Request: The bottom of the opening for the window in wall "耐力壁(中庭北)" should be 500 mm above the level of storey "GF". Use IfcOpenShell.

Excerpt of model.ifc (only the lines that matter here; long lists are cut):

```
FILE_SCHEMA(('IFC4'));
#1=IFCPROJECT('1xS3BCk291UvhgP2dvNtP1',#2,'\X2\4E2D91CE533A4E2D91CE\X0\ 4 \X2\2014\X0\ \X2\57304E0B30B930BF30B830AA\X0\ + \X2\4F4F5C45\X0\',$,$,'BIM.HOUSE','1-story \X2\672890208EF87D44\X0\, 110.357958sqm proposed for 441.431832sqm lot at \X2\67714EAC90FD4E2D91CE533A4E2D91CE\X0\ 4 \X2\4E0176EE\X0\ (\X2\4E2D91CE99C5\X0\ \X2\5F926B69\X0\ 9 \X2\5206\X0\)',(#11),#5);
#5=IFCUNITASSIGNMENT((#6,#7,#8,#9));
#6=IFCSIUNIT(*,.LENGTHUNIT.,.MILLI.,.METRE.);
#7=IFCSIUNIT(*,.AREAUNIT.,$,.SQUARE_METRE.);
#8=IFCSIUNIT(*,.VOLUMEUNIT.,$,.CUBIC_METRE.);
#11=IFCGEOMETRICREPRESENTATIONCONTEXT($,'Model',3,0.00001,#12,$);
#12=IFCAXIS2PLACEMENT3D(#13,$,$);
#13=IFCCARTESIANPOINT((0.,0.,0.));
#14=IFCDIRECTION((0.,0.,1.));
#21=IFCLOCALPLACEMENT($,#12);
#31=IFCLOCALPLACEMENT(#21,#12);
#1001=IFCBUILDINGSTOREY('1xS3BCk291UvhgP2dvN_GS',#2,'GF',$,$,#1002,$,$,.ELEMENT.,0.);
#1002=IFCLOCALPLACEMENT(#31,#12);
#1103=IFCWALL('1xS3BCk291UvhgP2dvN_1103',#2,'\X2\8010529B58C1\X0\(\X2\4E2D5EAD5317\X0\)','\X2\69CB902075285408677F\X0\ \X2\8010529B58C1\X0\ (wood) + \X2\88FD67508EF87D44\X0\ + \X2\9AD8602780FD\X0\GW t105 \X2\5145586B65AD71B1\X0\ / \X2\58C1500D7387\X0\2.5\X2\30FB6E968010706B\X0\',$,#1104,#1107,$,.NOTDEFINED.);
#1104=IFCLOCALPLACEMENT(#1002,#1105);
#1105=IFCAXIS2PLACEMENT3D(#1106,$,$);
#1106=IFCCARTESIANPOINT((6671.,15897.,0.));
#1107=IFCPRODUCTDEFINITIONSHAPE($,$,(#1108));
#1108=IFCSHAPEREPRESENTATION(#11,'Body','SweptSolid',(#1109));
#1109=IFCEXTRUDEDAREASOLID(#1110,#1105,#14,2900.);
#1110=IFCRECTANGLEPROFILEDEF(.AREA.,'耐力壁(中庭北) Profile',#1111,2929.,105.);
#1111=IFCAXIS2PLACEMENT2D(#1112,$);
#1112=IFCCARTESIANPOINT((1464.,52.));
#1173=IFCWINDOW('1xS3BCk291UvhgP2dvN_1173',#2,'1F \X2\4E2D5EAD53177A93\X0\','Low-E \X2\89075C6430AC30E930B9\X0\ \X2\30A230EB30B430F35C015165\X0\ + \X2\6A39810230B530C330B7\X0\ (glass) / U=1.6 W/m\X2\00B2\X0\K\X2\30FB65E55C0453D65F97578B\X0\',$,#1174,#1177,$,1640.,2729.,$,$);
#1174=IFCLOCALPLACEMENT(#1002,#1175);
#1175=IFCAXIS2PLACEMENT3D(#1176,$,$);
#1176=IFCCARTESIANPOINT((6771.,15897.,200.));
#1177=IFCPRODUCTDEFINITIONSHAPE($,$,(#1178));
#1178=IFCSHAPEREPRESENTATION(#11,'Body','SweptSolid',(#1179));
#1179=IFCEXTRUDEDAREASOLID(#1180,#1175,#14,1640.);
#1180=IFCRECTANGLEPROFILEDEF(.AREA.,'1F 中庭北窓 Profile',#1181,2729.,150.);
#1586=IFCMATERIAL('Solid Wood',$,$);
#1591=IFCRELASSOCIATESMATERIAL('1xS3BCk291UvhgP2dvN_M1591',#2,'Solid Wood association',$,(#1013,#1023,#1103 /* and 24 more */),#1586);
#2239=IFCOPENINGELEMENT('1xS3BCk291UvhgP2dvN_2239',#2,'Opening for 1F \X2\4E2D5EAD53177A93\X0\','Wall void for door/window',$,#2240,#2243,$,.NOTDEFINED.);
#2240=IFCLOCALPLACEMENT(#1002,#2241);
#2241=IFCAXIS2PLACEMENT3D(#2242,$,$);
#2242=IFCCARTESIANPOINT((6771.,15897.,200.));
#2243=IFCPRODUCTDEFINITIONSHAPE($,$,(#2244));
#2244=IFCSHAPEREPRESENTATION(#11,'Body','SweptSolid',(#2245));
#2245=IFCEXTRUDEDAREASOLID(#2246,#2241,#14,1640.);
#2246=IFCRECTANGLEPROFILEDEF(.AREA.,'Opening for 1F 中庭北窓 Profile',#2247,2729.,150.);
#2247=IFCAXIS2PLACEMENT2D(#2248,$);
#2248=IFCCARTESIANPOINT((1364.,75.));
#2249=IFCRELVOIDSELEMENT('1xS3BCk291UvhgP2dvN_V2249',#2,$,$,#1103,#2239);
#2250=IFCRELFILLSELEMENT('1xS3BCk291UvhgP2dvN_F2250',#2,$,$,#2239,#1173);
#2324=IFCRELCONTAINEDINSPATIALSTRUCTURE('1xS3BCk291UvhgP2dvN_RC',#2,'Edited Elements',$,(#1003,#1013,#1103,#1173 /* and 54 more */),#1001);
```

```python
import numpy as np
import ifcopenshell
import ifcopenshell.api.geometry
import ifcopenshell.geom
import ifcopenshell.util.element
import ifcopenshell.util.placement
import ifcopenshell.util.shape
import ifcopenshell.util.unit

model = ifcopenshell.open("model.ifc")
unit_scale = ifcopenshell.util.unit.calculate_unit_scale(model)

window = model.by_guid("1xS3BCk291UvhgP2dvN_1173")
opening = window.FillsVoids[0].RelatingOpeningElement
storey = ifcopenshell.util.element.get_container(window, ifc_class="IfcBuildingStorey")
level = ifcopenshell.util.placement.get_local_placement(storey.ObjectPlacement)[2, 3]

# The opening's origin need not be at the sill, so measure its lowest point.
shape = ifcopenshell.geom.create_shape(ifcopenshell.geom.settings(), opening)
bottom = ifcopenshell.util.shape.get_shape_bottom_elevation(shape, shape.geometry) / unit_scale
dz = level + 0.5 / unit_scale - bottom

shift = np.array([0.0, 0.0, dz])
# The window is not placed relative to its opening, so move both.
for product in (opening, window):
    matrix = ifcopenshell.util.placement.get_local_placement(product.ObjectPlacement)
    matrix[:3, 3] += shift
    ifcopenshell.api.geometry.edit_object_placement(model, product=product, matrix=matrix, is_si=False)

print(f"moved by {dz * unit_scale:+.3f} m")

model.write("model_v2.ifc")
```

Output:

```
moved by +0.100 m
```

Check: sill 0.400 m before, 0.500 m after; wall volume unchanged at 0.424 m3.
